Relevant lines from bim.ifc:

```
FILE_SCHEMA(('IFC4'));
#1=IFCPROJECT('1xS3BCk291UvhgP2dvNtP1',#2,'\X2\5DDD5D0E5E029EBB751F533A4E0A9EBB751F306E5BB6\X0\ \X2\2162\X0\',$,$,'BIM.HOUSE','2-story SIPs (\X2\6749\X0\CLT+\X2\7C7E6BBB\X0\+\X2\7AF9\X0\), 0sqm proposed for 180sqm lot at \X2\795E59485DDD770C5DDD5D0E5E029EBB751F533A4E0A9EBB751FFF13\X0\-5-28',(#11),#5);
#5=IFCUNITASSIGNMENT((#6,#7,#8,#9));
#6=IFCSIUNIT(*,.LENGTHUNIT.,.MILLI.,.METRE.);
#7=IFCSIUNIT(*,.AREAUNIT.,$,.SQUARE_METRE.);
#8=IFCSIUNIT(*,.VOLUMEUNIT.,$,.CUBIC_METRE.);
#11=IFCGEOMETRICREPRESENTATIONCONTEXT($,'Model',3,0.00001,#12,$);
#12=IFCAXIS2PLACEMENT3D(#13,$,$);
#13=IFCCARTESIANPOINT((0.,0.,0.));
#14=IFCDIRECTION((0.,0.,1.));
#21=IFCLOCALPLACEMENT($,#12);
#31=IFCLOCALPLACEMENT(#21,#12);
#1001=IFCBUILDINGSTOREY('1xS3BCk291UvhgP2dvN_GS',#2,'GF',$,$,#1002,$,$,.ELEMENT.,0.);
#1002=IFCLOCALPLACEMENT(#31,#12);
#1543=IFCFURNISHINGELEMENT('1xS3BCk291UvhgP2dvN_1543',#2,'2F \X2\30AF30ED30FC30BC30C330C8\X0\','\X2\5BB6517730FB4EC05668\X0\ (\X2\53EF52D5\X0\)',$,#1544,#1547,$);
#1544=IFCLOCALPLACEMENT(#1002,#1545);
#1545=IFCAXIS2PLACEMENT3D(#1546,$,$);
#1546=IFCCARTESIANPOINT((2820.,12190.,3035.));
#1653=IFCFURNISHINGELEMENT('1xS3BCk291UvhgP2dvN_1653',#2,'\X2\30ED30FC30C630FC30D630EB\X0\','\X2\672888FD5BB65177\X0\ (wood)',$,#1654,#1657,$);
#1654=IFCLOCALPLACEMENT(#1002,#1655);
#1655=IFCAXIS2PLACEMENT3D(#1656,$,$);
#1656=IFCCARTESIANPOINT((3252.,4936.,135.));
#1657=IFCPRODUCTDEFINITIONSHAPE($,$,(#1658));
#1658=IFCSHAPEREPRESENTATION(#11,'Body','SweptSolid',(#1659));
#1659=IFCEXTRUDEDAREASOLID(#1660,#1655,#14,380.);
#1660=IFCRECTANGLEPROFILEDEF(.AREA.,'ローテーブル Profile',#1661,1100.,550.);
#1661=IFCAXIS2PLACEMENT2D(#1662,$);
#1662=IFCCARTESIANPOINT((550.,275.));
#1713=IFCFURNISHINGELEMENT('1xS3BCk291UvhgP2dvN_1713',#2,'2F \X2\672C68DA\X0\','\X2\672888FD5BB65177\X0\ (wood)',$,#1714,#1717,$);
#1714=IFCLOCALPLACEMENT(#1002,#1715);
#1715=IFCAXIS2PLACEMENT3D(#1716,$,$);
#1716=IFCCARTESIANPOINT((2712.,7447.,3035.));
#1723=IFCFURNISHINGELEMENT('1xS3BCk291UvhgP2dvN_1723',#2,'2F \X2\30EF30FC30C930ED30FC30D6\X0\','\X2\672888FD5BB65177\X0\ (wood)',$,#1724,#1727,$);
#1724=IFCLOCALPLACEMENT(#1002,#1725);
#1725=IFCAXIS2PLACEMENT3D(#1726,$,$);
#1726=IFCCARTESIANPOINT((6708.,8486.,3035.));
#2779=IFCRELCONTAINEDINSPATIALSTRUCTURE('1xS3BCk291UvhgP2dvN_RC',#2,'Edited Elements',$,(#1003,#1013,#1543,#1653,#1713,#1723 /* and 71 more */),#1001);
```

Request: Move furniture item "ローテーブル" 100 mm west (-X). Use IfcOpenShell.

```python
import ifcopenshell
import ifcopenshell.api.geometry
import ifcopenshell.util.placement

model = ifcopenshell.open("bim.ifc")

item = model.by_guid("1xS3BCk291UvhgP2dvN_1653")
matrix = ifcopenshell.util.placement.get_local_placement(item.ObjectPlacement)
matrix[0, 3] -= 100.0
ifcopenshell.api.geometry.edit_object_placement(model, product=item, matrix=matrix, is_si=False)

print(ifcopenshell.util.placement.get_local_placement(item.ObjectPlacement).round(3) + 0.0)

model.write("bim_v2.ifc")
```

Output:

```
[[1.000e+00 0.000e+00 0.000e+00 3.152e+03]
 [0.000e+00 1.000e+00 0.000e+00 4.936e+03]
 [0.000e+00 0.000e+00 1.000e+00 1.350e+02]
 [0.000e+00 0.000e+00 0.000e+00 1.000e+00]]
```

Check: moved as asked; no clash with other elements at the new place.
